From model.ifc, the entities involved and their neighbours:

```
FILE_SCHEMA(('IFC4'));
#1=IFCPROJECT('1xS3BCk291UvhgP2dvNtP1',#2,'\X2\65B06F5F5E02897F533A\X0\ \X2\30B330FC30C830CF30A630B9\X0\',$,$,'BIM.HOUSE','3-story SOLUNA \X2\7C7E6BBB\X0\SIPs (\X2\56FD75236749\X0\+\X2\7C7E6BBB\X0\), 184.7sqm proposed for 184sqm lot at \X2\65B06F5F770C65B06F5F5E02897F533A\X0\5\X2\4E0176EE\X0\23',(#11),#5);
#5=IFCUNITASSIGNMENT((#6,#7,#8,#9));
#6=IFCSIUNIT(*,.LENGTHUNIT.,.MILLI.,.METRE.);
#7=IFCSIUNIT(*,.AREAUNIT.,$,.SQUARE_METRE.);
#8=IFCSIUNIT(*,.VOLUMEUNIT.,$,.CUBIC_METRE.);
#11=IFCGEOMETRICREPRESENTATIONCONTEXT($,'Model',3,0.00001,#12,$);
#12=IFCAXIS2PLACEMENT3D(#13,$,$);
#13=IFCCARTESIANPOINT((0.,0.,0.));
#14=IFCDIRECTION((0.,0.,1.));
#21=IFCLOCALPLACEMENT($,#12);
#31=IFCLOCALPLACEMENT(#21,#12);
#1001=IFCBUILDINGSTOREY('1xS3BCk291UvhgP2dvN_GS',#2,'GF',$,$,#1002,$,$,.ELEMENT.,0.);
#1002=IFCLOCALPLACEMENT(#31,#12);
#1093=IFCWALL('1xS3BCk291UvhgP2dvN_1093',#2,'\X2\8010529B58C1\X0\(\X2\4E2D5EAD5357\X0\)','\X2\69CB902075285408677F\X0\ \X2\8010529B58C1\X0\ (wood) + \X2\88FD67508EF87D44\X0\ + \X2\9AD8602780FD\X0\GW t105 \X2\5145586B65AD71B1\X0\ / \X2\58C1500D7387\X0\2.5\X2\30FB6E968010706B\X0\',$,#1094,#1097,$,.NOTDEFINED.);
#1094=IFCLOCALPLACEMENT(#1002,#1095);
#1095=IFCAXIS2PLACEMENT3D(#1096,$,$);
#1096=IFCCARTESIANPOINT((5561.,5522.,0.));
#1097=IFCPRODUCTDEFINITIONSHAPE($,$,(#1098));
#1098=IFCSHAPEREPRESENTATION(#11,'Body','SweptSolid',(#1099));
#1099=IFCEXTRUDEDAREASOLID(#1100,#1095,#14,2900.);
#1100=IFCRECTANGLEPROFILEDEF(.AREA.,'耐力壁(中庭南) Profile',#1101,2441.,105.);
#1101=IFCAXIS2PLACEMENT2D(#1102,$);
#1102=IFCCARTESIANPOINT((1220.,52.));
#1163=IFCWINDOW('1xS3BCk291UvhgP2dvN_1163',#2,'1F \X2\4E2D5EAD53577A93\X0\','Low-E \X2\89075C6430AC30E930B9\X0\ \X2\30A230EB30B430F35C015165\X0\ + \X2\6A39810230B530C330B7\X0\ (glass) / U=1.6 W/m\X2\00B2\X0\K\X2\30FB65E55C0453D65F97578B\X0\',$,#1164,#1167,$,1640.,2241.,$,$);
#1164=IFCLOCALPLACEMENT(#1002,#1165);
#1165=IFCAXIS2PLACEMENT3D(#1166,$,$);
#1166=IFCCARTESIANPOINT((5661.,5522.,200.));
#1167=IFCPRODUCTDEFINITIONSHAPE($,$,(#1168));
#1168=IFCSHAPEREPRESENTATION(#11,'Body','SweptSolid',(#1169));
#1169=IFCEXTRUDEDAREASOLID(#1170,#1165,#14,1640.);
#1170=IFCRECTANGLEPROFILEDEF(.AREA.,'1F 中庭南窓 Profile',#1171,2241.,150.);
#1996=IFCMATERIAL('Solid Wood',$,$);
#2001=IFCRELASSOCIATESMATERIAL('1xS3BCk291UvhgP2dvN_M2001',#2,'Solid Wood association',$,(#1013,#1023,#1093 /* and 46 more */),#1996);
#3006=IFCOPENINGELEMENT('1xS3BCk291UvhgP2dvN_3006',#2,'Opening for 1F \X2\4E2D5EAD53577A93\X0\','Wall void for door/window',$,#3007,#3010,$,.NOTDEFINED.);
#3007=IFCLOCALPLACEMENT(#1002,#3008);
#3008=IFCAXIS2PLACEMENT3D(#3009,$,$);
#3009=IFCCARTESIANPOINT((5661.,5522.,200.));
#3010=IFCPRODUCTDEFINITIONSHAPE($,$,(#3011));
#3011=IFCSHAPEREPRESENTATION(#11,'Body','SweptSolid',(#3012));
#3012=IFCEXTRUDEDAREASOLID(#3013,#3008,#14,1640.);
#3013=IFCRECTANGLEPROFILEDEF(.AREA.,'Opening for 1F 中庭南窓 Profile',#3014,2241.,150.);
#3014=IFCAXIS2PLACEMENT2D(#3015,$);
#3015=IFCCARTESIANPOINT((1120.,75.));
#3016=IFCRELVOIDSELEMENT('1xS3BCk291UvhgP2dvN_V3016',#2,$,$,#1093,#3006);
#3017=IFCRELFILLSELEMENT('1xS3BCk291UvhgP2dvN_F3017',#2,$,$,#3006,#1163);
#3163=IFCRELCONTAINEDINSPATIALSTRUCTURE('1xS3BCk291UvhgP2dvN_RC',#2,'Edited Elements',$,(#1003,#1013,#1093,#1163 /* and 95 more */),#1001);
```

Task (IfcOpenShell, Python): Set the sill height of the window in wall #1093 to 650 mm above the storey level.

```python
import numpy as np
import ifcopenshell
import ifcopenshell.api.geometry
import ifcopenshell.geom
import ifcopenshell.util.element
import ifcopenshell.util.placement
import ifcopenshell.util.shape
import ifcopenshell.util.unit

model = ifcopenshell.open("model.ifc")
unit_scale = ifcopenshell.util.unit.calculate_unit_scale(model)

window = model.by_id(1163)
opening = window.FillsVoids[0].RelatingOpeningElement
storey = ifcopenshell.util.element.get_container(window, ifc_class="IfcBuildingStorey")
level = ifcopenshell.util.placement.get_local_placement(storey.ObjectPlacement)[2, 3]

# The opening's origin need not be at the sill, so measure its lowest point.
shape = ifcopenshell.geom.create_shape(ifcopenshell.geom.settings(), opening)
bottom = ifcopenshell.util.shape.get_shape_bottom_elevation(shape, shape.geometry) / unit_scale
dz = level + 650.0 - bottom

shift = np.array([0.0, 0.0, dz])
# The window is not placed relative to its opening, so move both.
for product in (opening, window):
    matrix = ifcopenshell.util.placement.get_local_placement(product.ObjectPlacement)
    matrix[:3, 3] += shift
    ifcopenshell.api.geometry.edit_object_placement(model, product=product, matrix=matrix, is_si=False)

print(f"moved by {dz * unit_scale:+.3f} m")

model.write("model_rev.ifc")
```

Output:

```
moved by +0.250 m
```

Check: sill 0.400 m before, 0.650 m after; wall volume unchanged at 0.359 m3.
